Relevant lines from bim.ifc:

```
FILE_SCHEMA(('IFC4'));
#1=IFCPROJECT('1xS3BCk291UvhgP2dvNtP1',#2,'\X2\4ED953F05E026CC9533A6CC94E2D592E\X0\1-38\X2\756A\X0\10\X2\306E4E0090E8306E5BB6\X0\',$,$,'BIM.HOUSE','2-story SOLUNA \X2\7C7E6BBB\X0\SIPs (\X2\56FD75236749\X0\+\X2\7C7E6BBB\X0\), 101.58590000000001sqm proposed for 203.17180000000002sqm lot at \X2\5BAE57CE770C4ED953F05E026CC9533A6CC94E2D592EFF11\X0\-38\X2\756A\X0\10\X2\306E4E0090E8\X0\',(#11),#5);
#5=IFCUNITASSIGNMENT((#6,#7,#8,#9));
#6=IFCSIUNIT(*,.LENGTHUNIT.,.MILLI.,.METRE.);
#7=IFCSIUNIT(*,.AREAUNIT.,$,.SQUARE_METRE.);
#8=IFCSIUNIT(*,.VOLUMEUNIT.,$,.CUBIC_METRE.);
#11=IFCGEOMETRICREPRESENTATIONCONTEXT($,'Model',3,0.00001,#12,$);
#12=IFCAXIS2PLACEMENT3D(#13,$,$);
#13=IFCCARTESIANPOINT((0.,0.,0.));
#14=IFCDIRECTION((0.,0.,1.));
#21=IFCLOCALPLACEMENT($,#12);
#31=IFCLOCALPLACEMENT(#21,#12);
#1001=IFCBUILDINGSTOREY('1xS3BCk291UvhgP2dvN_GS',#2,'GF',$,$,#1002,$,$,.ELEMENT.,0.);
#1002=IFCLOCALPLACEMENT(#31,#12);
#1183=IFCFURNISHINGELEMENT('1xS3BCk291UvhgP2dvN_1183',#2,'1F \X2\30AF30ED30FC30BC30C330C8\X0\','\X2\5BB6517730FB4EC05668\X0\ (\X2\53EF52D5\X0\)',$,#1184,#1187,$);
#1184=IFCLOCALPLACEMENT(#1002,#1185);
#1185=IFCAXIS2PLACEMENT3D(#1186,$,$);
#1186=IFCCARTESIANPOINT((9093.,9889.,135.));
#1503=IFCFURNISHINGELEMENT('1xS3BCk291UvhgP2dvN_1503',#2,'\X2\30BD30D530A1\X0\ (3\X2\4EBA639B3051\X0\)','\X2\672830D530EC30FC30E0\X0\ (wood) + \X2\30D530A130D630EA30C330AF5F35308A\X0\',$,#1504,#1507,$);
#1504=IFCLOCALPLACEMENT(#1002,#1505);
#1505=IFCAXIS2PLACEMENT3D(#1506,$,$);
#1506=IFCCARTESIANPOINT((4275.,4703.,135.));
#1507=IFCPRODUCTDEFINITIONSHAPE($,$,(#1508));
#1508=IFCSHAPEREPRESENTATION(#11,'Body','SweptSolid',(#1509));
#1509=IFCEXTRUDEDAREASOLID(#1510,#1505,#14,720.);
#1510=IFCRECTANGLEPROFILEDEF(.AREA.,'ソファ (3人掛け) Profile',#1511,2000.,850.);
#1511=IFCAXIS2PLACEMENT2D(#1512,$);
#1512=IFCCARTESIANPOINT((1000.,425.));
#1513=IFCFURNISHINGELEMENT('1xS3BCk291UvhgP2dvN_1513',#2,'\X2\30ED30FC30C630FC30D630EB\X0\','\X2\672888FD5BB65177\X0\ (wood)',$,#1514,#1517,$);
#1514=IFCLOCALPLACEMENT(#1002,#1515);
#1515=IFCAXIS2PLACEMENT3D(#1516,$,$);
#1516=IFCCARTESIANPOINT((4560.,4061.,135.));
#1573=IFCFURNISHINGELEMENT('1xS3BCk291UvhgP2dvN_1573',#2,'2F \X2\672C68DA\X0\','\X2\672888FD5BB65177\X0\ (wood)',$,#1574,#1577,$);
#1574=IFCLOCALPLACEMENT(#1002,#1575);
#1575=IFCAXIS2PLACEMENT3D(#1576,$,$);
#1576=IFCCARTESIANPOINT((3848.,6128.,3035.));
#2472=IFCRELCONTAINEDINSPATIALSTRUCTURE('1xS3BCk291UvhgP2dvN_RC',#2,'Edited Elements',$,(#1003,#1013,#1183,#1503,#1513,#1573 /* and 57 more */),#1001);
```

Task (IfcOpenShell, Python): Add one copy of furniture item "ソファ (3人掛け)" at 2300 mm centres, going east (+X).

```python
import numpy as np
import ifcopenshell
import ifcopenshell.api.geometry
import ifcopenshell.api.root
import ifcopenshell.util.element
import ifcopenshell.util.placement
import ifcopenshell.util.unit

model = ifcopenshell.open("bim.ifc")
unit_scale = ifcopenshell.util.unit.calculate_unit_scale(model)


def reuse_history(source, copy):
    """copy_class also copies each property set's owner history, people and application; keep the originals."""
    for rel in copy.IsDefinedBy:
        if rel.is_a("IfcRelDefinesByProperties") and (history := rel.RelatingPropertyDefinition.OwnerHistory):
            rel.RelatingPropertyDefinition.OwnerHistory = source.OwnerHistory
            ifcopenshell.util.element.remove_deep2(model, history)


source = model.by_id(1503)
base = ifcopenshell.util.placement.get_local_placement(source.ObjectPlacement)
step = np.array([1.0, 0.0, 0.0]) * 2.3 / unit_scale

for i in range(1, 2):
    copy = ifcopenshell.api.root.copy_class(model, product=source)
    copy.Representation = ifcopenshell.util.element.copy_deep(
        model, source.Representation, exclude=["IfcGeometricRepresentationContext", "IfcRepresentationMap"]
    )
    reuse_history(source, copy)
    matrix = base.copy()
    matrix[:3, 3] += i * step
    print("added at", matrix[:3, 3].round(3) + 0.0)
    ifcopenshell.api.geometry.edit_object_placement(model, product=copy, matrix=matrix, is_si=False)

model.write("bim_rev.ifc")
```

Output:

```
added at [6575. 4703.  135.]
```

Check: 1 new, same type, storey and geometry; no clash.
